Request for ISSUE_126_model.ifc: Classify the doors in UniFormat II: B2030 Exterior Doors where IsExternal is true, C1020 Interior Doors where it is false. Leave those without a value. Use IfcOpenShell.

First a look at what the model holds.

```python
import ifcopenshell
import ifcopenshell.util.element

model = ifcopenshell.open("ISSUE_126_model.ifc")
print(model.schema)
print("classifications:", [c.Name for c in model.by_type("IfcClassification")])
values = [ifcopenshell.util.element.get_pset(e, "Pset_DoorCommon", "IsExternal") for e in model.by_type("IfcDoor")]
for value in (True, False, None):
    print("IsExternal", value, values.count(value))
```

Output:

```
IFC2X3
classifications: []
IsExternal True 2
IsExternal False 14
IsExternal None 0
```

```python
import ifcopenshell
import ifcopenshell.api.classification
import ifcopenshell.util.element

model = ifcopenshell.open("ISSUE_126_model.ifc")

# IFC2X3 requires Source and Edition and has no link from the project to the system.
system = model.create_entity("IfcClassification", Source="ASTM", Edition="E1557", Name="UniFormat II")

doors = model.by_type("IfcDoor")
external = {e: ifcopenshell.util.element.get_pset(e, "Pset_DoorCommon", "IsExternal") for e in doors}
for flag, code, name in ((True, "B2030", "Exterior Doors"), (False, "C1020", "Interior Doors")):
    products = [e for e in doors if external[e] is flag]
    ifcopenshell.api.classification.add_reference(
        model, products=products, classification=system, identification=code, name=name
    )
    print(code, len(products))

model.write("ISSUE_126_model_updated.ifc")
```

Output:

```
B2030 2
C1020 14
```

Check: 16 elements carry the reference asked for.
